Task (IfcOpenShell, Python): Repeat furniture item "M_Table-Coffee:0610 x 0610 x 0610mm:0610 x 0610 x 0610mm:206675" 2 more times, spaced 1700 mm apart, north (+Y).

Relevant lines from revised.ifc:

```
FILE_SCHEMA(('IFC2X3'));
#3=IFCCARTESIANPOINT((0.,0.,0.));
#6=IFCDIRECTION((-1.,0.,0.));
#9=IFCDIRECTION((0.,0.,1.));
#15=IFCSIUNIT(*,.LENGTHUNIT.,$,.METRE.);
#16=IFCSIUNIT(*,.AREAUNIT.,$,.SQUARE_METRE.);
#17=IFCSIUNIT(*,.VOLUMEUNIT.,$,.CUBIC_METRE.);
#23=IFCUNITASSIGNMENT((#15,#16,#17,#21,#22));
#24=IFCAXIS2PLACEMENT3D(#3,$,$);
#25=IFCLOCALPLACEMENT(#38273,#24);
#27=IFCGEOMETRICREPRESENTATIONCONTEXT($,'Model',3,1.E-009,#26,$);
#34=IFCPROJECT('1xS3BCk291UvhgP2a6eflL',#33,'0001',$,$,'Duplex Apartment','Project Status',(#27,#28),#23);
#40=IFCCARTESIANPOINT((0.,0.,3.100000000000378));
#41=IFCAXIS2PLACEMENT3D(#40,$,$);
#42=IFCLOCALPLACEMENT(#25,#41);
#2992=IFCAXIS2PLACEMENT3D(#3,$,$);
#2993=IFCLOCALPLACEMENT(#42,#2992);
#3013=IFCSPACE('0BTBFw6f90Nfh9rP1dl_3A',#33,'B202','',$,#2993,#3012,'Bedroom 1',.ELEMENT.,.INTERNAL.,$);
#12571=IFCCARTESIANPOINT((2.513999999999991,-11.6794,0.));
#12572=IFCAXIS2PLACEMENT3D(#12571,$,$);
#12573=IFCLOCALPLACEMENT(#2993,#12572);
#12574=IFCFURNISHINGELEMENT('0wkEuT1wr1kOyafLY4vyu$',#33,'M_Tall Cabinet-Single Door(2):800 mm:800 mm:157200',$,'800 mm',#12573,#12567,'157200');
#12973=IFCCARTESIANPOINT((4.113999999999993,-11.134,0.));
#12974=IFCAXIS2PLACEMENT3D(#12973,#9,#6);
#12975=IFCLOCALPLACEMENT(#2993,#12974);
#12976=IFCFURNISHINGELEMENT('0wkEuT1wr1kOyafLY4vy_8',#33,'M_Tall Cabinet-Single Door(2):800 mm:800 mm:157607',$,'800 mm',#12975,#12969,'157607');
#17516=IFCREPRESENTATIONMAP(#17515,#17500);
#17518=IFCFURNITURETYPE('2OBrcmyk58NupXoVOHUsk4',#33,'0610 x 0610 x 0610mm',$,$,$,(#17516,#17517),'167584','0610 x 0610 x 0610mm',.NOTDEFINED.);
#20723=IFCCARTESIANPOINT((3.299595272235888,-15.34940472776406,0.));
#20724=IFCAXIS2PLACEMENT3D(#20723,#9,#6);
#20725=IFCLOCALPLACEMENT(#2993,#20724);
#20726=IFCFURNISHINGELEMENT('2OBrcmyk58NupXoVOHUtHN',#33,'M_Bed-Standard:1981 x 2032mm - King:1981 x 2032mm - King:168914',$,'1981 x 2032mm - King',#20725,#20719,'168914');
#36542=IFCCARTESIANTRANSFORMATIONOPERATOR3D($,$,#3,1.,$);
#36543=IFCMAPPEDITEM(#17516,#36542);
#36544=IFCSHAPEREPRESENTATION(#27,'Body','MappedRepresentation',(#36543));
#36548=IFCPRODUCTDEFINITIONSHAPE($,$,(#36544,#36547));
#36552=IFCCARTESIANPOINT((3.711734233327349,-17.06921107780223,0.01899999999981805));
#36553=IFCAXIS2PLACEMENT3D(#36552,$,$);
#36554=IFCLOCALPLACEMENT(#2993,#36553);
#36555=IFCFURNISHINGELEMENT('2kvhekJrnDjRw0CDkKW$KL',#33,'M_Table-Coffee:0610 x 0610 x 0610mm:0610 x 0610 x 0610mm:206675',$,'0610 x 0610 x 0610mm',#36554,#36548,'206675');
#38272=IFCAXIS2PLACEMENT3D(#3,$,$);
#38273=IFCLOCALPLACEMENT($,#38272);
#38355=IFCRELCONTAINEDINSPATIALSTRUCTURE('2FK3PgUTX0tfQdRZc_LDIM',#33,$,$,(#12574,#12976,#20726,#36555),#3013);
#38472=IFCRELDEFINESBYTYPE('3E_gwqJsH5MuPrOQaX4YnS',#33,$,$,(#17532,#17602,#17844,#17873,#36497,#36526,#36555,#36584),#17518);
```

```python
import numpy as np
import ifcopenshell
import ifcopenshell.api.geometry
import ifcopenshell.api.root
import ifcopenshell.util.element
import ifcopenshell.util.placement
import ifcopenshell.util.unit

model = ifcopenshell.open("revised.ifc")
unit_scale = ifcopenshell.util.unit.calculate_unit_scale(model)


def reuse_history(source, copy):
    """copy_class also copies each property set's owner history, people and application; keep the originals."""
    for rel in copy.IsDefinedBy:
        if rel.is_a("IfcRelDefinesByProperties") and (history := rel.RelatingPropertyDefinition.OwnerHistory):
            rel.RelatingPropertyDefinition.OwnerHistory = source.OwnerHistory
            ifcopenshell.util.element.remove_deep2(model, history)


source = model.by_guid("2kvhekJrnDjRw0CDkKW$KL")
base = ifcopenshell.util.placement.get_local_placement(source.ObjectPlacement)
step = np.array([0.0, 1.0, 0.0]) * 1.7 / unit_scale

for i in range(1, 3):
    copy = ifcopenshell.api.root.copy_class(model, product=source)
    copy.Representation = ifcopenshell.util.element.copy_deep(
        model, source.Representation, exclude=["IfcGeometricRepresentationContext", "IfcRepresentationMap"]
    )
    copy.Name = "M_Table-Coffee:0610 x 0610 x 0610mm:0610 x 0610 x 0610mm"
    copy.Tag = None
    reuse_history(source, copy)
    matrix = base.copy()
    matrix[:3, 3] += i * step
    print("added at", matrix[:3, 3].round(3) + 0.0)
    ifcopenshell.api.geometry.edit_object_placement(model, product=copy, matrix=matrix, is_si=False)

model.write("revised_edited.ifc")
```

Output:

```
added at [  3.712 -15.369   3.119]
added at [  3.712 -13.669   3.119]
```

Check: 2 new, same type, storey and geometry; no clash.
